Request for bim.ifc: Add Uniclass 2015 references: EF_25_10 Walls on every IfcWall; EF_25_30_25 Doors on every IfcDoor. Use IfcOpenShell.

First a look at what the model holds.

```python
import ifcopenshell

model = ifcopenshell.open("bim.ifc")
print(model.schema)
print("classifications:", [c.Name for c in model.by_type("IfcClassification")])
for ifc_class in ("IfcDoor", "IfcRoof", "IfcStair", "IfcWall", "IfcWindow"):
    print(ifc_class, len(model.by_type(ifc_class)))
```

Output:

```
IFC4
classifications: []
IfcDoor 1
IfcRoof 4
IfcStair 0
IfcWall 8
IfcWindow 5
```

```python
import ifcopenshell
import ifcopenshell.api.classification

model = ifcopenshell.open("bim.ifc")

system = ifcopenshell.api.classification.add_classification(model, classification="Uniclass 2015")

codes = {
    "IfcWall": ("EF_25_10", "Walls"),
    "IfcDoor": ("EF_25_30_25", "Doors"),
}
for ifc_class, (code, name) in codes.items():
    products = model.by_type(ifc_class)
    ifcopenshell.api.classification.add_reference(
        model, products=products, classification=system, identification=code, name=name
    )
    print(code, len(products))

model.write("bim-out.ifc")
```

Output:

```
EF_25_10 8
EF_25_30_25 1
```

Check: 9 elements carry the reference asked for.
